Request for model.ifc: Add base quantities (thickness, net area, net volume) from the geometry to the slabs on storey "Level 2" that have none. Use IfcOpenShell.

First a look at what the model holds.

```python
import ifcopenshell
import ifcopenshell.util.element
import ifcopenshell.util.unit

model = ifcopenshell.open("model.ifc")
print(model.schema)
for unit_type in ("LENGTHUNIT", "AREAUNIT", "VOLUMEUNIT"):
    print(unit_type, ifcopenshell.util.unit.calculate_unit_scale(model, unit_type))
storey = next(s for s in model.by_type("IfcBuildingStorey") if s.Name == "Level 2")
slabs = [e for e in ifcopenshell.util.element.get_decomposition(storey) if e.is_a("IfcSlab")]
for e in sorted(slabs, key=lambda e: e.id()):
    print(e.id(), e.is_a(), e.Name, list(ifcopenshell.util.element.get_psets(e, qtos_only=True)), sep=" | ")
```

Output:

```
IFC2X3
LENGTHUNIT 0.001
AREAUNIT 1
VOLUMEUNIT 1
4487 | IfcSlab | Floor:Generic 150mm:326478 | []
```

```python
import ifcopenshell
import ifcopenshell.api.pset
import ifcopenshell.geom
import ifcopenshell.util.element
import ifcopenshell.util.shape
import ifcopenshell.util.unit

model = ifcopenshell.open("model.ifc")
unit_scale = ifcopenshell.util.unit.calculate_unit_scale(model)
area_scale = ifcopenshell.util.unit.calculate_unit_scale(model, "AREAUNIT")
volume_scale = ifcopenshell.util.unit.calculate_unit_scale(model, "VOLUMEUNIT")
settings = ifcopenshell.geom.settings()

storey = next(s for s in model.by_type("IfcBuildingStorey") if s.Name == "Level 2")
slabs = [e for e in ifcopenshell.util.element.get_decomposition(storey) if e.is_a("IfcSlab")]

for e in sorted(slabs, key=lambda e: e.id()):
    if ifcopenshell.util.element.get_psets(e, qtos_only=True, should_inherit=False):
        continue
    # Geometry comes back in metres, in the element's own axes.
    shape = ifcopenshell.geom.create_shape(settings, e)
    values = {
        "Width": ifcopenshell.util.shape.get_z(shape.geometry) / unit_scale,
        "NetArea": ifcopenshell.util.shape.get_footprint_area(shape.geometry) / area_scale,
        "NetVolume": ifcopenshell.util.shape.get_volume(shape.geometry) / volume_scale,
    }
    qto = ifcopenshell.api.pset.add_qto(model, product=e, name="BaseQuantities")
    ifcopenshell.api.pset.edit_qto(model, qto=qto, properties=values)
    print(e.id(), {k: round(v, 3) for k, v in values.items()})

model.write("model-out.ifc")
```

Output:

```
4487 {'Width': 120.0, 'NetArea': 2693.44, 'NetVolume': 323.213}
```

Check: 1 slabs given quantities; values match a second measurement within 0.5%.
